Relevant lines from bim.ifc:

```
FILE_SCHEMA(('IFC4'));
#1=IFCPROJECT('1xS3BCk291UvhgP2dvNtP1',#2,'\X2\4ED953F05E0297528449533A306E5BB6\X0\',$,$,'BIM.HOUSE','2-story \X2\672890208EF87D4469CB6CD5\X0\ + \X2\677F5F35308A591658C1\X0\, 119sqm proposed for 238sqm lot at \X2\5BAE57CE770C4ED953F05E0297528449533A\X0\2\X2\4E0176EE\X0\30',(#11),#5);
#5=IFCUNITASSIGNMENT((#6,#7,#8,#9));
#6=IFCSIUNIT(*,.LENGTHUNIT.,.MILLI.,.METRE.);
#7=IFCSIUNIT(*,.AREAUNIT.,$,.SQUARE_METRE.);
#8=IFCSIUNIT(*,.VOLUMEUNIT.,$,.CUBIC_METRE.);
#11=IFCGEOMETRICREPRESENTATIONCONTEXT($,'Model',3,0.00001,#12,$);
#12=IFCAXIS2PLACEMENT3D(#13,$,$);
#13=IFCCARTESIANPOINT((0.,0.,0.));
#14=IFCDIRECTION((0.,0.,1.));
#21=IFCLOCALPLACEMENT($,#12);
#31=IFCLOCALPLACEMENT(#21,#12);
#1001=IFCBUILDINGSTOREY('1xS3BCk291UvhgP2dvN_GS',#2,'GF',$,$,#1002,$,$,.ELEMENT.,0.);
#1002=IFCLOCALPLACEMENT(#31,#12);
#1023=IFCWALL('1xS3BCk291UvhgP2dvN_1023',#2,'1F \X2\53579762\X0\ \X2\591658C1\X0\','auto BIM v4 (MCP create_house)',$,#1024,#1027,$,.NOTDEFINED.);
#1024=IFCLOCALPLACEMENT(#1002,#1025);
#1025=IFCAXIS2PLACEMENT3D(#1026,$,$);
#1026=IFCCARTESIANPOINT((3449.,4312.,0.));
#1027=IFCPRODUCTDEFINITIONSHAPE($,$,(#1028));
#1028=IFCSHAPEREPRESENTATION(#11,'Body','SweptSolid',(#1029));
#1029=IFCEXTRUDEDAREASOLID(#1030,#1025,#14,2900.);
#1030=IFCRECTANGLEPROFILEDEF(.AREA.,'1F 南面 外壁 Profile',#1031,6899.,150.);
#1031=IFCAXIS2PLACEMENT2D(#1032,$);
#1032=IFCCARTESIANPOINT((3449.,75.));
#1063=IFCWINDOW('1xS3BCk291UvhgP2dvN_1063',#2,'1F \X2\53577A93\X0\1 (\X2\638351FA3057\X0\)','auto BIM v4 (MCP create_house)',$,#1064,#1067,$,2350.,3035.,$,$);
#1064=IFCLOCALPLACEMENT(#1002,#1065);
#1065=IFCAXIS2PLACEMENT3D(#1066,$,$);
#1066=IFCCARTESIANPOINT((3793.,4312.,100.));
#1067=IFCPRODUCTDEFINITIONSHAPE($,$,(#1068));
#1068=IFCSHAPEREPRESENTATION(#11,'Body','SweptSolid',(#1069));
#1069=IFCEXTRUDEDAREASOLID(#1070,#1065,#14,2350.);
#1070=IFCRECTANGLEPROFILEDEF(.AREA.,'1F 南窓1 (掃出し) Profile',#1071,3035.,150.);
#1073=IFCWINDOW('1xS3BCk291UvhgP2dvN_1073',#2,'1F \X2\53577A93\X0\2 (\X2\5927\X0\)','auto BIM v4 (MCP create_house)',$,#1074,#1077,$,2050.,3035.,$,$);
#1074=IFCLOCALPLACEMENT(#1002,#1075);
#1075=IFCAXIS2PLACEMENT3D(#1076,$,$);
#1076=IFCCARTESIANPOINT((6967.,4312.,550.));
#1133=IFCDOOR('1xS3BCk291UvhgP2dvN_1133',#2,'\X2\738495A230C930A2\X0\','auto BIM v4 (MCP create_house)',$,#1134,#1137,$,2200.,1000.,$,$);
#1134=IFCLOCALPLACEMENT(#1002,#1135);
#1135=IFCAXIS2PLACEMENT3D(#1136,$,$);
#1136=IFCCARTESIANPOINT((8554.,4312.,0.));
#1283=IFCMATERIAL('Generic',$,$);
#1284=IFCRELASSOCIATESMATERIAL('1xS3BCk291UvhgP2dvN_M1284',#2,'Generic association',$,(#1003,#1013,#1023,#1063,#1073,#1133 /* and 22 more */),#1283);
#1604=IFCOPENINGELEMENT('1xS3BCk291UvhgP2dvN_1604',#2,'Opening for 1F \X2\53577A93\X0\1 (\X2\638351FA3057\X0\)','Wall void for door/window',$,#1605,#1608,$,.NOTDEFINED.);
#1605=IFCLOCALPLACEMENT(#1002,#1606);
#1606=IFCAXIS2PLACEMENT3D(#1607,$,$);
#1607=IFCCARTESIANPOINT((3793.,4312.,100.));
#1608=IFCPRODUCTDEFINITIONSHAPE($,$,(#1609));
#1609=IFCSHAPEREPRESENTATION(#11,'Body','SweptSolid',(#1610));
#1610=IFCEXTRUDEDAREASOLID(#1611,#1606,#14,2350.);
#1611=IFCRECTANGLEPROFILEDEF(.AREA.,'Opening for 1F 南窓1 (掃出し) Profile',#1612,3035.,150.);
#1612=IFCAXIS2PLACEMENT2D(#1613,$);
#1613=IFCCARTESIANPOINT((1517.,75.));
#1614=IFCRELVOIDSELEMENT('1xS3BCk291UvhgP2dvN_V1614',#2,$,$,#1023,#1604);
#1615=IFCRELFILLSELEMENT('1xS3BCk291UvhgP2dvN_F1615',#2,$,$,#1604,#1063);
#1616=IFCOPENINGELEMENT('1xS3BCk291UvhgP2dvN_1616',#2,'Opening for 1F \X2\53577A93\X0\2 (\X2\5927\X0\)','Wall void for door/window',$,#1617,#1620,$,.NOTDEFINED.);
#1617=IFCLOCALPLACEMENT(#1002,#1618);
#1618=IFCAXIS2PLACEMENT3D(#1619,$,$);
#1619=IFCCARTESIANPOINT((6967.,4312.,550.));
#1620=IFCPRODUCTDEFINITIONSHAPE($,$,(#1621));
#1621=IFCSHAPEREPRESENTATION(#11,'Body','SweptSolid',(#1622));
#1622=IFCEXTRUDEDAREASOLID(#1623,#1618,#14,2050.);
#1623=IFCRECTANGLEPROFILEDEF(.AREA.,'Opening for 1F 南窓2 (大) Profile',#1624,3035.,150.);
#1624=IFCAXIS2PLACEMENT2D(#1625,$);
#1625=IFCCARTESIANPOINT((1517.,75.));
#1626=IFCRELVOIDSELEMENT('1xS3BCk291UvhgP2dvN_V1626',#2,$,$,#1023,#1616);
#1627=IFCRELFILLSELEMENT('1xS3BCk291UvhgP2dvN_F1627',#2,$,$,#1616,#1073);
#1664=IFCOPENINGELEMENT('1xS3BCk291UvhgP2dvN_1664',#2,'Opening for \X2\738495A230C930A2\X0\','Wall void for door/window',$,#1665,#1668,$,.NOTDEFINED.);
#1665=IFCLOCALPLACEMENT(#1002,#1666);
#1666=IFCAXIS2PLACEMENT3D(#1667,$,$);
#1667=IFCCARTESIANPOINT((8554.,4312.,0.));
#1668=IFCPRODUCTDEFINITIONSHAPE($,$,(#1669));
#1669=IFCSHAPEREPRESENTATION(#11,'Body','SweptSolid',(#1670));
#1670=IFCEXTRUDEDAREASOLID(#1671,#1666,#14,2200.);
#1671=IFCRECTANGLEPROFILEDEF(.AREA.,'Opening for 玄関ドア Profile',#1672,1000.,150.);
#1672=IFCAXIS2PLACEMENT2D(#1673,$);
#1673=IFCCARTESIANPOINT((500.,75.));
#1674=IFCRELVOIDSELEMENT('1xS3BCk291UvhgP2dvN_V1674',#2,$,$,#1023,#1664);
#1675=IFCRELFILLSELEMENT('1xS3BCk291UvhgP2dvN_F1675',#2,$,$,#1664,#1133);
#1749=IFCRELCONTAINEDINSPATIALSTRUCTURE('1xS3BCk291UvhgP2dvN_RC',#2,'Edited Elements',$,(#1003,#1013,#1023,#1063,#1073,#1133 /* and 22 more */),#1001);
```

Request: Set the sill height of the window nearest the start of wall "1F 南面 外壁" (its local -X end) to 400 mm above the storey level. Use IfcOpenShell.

```python
import numpy as np
import ifcopenshell
import ifcopenshell.api.geometry
import ifcopenshell.geom
import ifcopenshell.util.element
import ifcopenshell.util.placement
import ifcopenshell.util.shape
import ifcopenshell.util.unit

model = ifcopenshell.open("bim.ifc")
unit_scale = ifcopenshell.util.unit.calculate_unit_scale(model)

window = model.by_guid("1xS3BCk291UvhgP2dvN_1063")
opening = window.FillsVoids[0].RelatingOpeningElement
storey = ifcopenshell.util.element.get_container(window, ifc_class="IfcBuildingStorey")
level = ifcopenshell.util.placement.get_local_placement(storey.ObjectPlacement)[2, 3]

# The opening's origin need not be at the sill, so measure its lowest point.
shape = ifcopenshell.geom.create_shape(ifcopenshell.geom.settings(), opening)
bottom = ifcopenshell.util.shape.get_shape_bottom_elevation(shape, shape.geometry) / unit_scale
dz = level + 400.0 - bottom

shift = np.array([0.0, 0.0, dz])
# The window is not placed relative to its opening, so move both.
for product in (opening, window):
    matrix = ifcopenshell.util.placement.get_local_placement(product.ObjectPlacement)
    matrix[:3, 3] += shift
    ifcopenshell.api.geometry.edit_object_placement(model, product=product, matrix=matrix, is_si=False)

print(f"moved by {dz * unit_scale:+.3f} m")

model.write("bim_edited.ifc")
```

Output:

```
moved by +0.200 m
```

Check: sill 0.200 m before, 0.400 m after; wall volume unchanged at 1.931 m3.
